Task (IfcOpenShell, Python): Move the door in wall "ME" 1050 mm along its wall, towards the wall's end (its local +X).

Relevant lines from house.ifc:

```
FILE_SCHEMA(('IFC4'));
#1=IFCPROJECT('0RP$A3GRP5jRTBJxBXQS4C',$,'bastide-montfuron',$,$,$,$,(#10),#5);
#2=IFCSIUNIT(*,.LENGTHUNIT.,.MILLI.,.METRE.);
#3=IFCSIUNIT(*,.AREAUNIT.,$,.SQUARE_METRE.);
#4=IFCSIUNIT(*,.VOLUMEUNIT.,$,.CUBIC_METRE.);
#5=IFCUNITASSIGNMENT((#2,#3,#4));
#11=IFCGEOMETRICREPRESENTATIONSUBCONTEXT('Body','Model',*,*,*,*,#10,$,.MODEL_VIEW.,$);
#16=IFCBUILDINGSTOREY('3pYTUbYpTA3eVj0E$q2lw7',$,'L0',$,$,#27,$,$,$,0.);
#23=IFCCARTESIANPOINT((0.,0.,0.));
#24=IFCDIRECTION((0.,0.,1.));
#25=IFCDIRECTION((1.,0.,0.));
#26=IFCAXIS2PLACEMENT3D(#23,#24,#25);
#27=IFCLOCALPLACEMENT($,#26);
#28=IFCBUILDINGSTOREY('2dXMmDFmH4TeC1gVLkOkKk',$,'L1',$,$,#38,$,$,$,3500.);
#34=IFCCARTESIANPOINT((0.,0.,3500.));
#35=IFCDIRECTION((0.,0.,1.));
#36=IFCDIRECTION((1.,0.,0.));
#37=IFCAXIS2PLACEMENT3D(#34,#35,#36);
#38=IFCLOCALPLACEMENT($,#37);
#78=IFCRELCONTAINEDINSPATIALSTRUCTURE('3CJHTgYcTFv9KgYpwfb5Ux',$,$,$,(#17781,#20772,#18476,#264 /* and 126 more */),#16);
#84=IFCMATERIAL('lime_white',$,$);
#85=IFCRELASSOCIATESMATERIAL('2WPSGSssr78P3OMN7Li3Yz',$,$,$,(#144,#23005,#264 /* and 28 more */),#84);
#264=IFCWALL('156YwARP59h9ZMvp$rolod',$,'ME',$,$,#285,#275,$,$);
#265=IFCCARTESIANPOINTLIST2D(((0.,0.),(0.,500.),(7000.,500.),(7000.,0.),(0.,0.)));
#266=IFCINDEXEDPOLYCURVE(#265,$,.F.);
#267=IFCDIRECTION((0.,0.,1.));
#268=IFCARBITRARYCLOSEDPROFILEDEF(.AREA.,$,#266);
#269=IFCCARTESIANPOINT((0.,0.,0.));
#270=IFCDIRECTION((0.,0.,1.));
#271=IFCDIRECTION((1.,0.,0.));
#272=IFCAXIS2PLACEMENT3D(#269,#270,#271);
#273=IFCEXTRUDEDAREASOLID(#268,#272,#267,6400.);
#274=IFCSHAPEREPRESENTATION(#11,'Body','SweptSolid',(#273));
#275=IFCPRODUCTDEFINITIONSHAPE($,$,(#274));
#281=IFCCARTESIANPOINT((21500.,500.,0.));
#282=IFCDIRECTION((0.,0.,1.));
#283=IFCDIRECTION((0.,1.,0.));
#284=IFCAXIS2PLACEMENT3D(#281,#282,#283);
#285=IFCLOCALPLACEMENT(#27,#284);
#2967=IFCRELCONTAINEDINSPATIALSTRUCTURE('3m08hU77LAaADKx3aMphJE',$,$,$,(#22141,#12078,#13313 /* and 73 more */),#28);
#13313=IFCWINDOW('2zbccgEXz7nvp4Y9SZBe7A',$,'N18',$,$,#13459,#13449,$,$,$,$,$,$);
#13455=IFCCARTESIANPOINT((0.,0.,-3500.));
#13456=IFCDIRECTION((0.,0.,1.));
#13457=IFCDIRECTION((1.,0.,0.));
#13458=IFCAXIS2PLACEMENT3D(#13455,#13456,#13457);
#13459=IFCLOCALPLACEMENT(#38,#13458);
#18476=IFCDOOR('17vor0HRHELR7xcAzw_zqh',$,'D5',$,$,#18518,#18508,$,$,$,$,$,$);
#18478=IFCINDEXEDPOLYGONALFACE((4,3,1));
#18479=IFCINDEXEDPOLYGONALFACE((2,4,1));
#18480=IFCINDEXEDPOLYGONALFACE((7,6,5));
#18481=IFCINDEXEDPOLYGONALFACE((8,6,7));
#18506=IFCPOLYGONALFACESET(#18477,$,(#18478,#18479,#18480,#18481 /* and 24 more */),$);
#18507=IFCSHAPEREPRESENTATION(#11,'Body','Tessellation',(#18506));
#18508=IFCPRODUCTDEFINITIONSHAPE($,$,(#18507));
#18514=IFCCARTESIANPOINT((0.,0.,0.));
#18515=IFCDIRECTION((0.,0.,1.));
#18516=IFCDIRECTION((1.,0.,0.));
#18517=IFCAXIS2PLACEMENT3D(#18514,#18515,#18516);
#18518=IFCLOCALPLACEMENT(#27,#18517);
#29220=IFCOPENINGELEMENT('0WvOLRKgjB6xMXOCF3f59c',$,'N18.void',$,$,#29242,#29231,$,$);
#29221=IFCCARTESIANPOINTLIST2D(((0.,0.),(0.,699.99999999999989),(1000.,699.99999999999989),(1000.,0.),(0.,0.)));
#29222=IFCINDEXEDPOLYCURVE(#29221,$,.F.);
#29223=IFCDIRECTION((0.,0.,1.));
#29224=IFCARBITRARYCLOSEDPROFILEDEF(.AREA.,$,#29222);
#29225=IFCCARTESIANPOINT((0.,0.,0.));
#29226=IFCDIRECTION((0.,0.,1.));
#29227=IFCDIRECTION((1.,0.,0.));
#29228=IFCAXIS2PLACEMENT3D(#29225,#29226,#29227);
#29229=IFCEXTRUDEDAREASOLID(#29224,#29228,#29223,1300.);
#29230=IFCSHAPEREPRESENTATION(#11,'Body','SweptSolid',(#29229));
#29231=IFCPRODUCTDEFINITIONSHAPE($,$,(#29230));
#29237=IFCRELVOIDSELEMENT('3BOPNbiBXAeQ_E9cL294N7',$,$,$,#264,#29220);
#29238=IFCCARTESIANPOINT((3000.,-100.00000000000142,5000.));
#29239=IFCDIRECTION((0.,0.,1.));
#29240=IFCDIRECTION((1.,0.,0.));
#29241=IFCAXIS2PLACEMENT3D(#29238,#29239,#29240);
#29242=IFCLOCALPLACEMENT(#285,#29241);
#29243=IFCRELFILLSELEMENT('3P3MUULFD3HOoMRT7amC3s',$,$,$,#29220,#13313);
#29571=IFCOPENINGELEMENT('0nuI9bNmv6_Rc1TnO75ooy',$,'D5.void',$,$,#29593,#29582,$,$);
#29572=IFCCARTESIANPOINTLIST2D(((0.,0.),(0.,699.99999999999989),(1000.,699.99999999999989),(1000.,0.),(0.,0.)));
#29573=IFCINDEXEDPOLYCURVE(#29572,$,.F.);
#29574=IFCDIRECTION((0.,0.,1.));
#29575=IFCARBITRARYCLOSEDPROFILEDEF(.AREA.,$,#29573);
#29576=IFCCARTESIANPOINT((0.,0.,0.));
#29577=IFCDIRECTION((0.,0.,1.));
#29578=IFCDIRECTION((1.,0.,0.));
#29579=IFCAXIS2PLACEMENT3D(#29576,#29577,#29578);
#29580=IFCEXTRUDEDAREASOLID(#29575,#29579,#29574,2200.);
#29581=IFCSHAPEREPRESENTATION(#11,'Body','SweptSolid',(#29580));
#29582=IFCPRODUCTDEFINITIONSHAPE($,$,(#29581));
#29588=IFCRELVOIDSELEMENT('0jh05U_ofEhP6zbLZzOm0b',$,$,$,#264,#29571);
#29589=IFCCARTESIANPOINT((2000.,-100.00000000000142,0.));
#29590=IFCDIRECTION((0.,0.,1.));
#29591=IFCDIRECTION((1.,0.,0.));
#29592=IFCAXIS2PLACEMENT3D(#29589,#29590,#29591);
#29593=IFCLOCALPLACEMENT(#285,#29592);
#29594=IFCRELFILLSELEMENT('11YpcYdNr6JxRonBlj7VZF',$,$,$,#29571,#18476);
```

```python
import ifcopenshell
import ifcopenshell.api.geometry
import ifcopenshell.util.placement

model = ifcopenshell.open("house.ifc")

door = model.by_guid("17vor0HRHELR7xcAzw_zqh")
opening = door.FillsVoids[0].RelatingOpeningElement
wall = opening.VoidsElements[0].RelatingBuildingElement

wall_matrix = ifcopenshell.util.placement.get_local_placement(wall.ObjectPlacement)
shift = wall_matrix[:3, 0] * 1050.0
before = ifcopenshell.util.placement.get_local_placement(door.ObjectPlacement)[:3, 3].copy()

# The door is not placed relative to its opening, so move both.
for product in (opening, door):
    matrix = ifcopenshell.util.placement.get_local_placement(product.ObjectPlacement)
    matrix[:3, 3] += shift
    ifcopenshell.api.geometry.edit_object_placement(model, product=product, matrix=matrix, is_si=False)

after = ifcopenshell.util.placement.get_local_placement(door.ObjectPlacement)[:3, 3]
print("door moved by", (after - before).round(3) + 0.0)

model.write("house_edited.ifc")
```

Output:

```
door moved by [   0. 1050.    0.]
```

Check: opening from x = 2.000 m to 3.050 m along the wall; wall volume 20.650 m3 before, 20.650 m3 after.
